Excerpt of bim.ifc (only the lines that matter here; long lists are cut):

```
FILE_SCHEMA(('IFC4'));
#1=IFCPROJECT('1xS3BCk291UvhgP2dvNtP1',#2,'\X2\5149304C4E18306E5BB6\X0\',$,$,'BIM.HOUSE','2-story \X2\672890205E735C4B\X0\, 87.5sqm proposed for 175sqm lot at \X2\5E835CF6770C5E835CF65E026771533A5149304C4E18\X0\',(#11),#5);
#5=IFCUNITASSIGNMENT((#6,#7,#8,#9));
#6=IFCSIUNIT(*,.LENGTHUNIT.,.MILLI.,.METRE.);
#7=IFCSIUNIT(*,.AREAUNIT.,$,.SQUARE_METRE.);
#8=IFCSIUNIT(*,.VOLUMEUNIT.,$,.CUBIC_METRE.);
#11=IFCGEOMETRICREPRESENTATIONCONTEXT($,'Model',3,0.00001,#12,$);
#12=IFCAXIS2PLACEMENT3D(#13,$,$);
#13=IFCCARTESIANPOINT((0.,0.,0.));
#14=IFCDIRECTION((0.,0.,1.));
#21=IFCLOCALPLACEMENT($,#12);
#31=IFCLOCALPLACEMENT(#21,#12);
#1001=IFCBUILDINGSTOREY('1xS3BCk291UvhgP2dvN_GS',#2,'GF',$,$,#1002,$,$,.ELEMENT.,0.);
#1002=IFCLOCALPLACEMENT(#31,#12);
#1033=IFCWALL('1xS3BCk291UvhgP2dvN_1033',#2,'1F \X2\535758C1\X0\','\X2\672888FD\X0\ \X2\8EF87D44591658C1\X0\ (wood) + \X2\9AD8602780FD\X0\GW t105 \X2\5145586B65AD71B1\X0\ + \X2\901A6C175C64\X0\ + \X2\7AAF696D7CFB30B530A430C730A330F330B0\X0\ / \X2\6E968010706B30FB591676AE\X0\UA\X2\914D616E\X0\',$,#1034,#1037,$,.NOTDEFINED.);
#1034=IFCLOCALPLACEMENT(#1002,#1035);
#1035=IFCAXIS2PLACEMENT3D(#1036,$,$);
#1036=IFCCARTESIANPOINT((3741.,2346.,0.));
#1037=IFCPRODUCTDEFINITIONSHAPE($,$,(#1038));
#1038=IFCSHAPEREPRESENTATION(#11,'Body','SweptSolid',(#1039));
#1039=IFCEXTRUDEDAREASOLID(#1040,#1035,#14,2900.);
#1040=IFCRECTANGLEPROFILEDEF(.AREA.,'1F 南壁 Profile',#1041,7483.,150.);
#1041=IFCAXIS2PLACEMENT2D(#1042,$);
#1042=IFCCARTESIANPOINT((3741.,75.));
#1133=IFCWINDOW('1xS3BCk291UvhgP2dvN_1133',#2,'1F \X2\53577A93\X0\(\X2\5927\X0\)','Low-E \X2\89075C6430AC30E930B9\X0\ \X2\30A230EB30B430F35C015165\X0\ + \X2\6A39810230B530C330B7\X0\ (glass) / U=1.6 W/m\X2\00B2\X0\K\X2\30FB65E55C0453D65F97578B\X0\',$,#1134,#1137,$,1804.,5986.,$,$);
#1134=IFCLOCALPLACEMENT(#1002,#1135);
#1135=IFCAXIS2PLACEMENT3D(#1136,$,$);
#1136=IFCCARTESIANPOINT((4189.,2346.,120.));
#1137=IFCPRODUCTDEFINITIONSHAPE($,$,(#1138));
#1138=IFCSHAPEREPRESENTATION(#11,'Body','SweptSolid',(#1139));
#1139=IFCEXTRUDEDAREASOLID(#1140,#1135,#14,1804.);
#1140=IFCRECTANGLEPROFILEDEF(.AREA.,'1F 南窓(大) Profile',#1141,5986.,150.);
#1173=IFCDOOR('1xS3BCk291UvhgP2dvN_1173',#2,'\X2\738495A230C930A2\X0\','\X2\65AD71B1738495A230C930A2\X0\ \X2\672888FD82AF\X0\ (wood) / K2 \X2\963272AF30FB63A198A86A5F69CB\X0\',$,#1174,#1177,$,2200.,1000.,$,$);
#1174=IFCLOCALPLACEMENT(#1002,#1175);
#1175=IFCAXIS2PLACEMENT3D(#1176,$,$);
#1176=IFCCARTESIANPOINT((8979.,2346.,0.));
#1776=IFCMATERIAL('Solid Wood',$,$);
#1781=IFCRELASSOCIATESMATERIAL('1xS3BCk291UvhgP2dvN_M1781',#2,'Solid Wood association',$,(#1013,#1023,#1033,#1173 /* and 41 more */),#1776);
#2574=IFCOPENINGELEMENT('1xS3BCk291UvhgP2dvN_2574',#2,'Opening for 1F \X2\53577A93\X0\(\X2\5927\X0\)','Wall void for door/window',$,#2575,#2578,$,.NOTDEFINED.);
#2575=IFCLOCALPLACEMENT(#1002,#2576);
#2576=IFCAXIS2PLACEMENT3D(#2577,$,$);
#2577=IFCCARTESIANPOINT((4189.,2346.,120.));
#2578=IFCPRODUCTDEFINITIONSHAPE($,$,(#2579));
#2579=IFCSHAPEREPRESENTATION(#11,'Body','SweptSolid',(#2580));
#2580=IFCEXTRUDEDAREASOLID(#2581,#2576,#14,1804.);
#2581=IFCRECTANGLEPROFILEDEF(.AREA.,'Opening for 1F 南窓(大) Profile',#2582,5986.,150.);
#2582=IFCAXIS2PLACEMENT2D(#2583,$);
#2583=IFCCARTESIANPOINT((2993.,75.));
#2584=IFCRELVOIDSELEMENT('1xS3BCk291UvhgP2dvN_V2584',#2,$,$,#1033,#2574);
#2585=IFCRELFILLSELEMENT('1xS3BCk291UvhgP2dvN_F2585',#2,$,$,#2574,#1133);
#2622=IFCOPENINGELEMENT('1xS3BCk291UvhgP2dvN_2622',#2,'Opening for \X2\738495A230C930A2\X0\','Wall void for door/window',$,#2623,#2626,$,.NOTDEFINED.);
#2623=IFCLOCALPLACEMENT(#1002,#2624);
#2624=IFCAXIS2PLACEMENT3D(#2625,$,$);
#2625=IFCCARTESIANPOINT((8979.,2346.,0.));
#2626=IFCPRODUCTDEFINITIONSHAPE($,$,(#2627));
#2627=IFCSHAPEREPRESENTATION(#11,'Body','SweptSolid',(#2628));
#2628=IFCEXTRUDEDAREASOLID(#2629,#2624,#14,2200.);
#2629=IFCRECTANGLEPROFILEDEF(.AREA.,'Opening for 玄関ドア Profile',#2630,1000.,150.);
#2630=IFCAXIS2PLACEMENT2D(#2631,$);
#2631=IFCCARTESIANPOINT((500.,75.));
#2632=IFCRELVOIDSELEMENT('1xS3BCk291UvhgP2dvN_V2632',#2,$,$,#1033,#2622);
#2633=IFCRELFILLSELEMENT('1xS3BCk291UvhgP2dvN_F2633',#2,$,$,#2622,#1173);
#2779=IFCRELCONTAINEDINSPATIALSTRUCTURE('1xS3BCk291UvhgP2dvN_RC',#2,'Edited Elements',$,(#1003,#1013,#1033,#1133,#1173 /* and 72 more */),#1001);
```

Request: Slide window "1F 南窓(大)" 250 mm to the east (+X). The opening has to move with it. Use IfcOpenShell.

```python
import ifcopenshell
import ifcopenshell.api.geometry
import ifcopenshell.util.placement
import ifcopenshell.util.unit

model = ifcopenshell.open("bim.ifc")
unit_scale = ifcopenshell.util.unit.calculate_unit_scale(model)

window = model.by_guid("1xS3BCk291UvhgP2dvN_1133")
opening = window.FillsVoids[0].RelatingOpeningElement
wall = opening.VoidsElements[0].RelatingBuildingElement

wall_matrix = ifcopenshell.util.placement.get_local_placement(wall.ObjectPlacement)
shift = wall_matrix[:3, 0] * 0.25 / unit_scale
before = ifcopenshell.util.placement.get_local_placement(window.ObjectPlacement)[:3, 3].copy()

# The window is not placed relative to its opening, so move both.
for product in (opening, window):
    matrix = ifcopenshell.util.placement.get_local_placement(product.ObjectPlacement)
    matrix[:3, 3] += shift
    ifcopenshell.api.geometry.edit_object_placement(model, product=product, matrix=matrix, is_si=False)

after = ifcopenshell.util.placement.get_local_placement(window.ObjectPlacement)[:3, 3]
print("window moved by", (after - before).round(3) + 0.0)

model.write("bim_edited.ifc")
```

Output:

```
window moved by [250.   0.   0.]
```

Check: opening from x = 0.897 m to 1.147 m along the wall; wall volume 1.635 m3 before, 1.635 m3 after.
